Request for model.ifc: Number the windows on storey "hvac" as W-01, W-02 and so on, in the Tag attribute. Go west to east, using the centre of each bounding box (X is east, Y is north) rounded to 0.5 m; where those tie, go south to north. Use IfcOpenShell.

First a look at what the model holds.

```python
import ifcopenshell
import ifcopenshell.util.element
import ifcopenshell.util.placement

model = ifcopenshell.open("model.ifc")
print(model.schema)
storey = next(s for s in model.by_type("IfcBuildingStorey") if s.Name == "hvac")
windows = [e for e in ifcopenshell.util.element.get_decomposition(storey) if e.is_a("IfcWindow")]
for e in sorted(windows, key=lambda e: e.id()):
    origin = ifcopenshell.util.placement.get_local_placement(e.ObjectPlacement)[:3, 3]
    print(e.id(), e.Tag, e.Name, origin.round(2) + 0.0, sep=" | ")
```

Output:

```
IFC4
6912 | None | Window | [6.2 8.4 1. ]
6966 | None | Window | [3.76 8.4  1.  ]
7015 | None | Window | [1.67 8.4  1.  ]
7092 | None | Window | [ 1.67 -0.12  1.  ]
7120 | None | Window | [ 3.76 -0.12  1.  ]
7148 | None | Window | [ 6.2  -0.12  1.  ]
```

```python
import ifcopenshell
import ifcopenshell.geom
import ifcopenshell.util.element
import ifcopenshell.util.shape

model = ifcopenshell.open("model.ifc")
settings = ifcopenshell.geom.settings()
settings.set("use-world-coords", True)


def centre(element):
    shape = ifcopenshell.geom.create_shape(settings, element)
    return ifcopenshell.util.shape.get_bbox_centroid(shape.geometry)


storey = next(s for s in model.by_type("IfcBuildingStorey") if s.Name == "hvac")
windows = [e for e in ifcopenshell.util.element.get_decomposition(storey) if e.is_a("IfcWindow")]

# Insertion points can sit at a corner or the storey origin, so sort by the geometry (in metres).
centres = {e: centre(e) for e in windows}
windows.sort(key=lambda e: (round(centres[e][0] / 0.5), centres[e][1]))

for i, e in enumerate(windows, start=1):
    number = f"W-{i:02d}"
    e.Tag = number
    print(e.id(), number)

model.write("model_rev.ifc")
```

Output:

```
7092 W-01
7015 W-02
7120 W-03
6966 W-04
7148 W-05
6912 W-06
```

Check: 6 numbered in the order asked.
